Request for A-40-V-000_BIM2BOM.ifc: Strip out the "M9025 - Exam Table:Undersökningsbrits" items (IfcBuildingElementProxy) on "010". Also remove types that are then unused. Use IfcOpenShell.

First a look at what the model holds.

```python
import ifcopenshell
import ifcopenshell.util.element

model = ifcopenshell.open("A-40-V-000_BIM2BOM.ifc")
print(model.schema)
storey = next(s for s in model.by_type("IfcBuildingStorey") if s.Name == "010")
proxies = [e for e in ifcopenshell.util.element.get_decomposition(storey) if e.is_a("IfcBuildingElementProxy")]
seen = {}
for e in proxies:
    element_type = ifcopenshell.util.element.get_type(e)
    name = element_type.Name if element_type not in (None, e) else None
    seen[name] = seen.get(name, 0) + 1
for name, count in sorted(seen.items(), key=str):
    print(count, "x", name)
```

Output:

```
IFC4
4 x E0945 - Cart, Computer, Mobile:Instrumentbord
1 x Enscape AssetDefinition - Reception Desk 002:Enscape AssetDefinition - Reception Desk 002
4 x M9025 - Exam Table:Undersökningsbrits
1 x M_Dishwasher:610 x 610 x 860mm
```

```python
import ifcopenshell
import ifcopenshell.api.root
import ifcopenshell.util.element

model = ifcopenshell.open("A-40-V-000_BIM2BOM.ifc")

storey = next(s for s in model.by_type("IfcBuildingStorey") if s.Name == "010")
proxies = [e for e in ifcopenshell.util.element.get_decomposition(storey) if e.is_a("IfcBuildingElementProxy")]
targets = [e for e in proxies if (t := ifcopenshell.util.element.get_type(e)) not in (None, e) and t.Name == "M9025 - Exam Table:Undersökningsbrits"]
types = {ifcopenshell.util.element.get_type(e) for e in targets} - {None, *targets}

for e in targets:
    ifcopenshell.api.root.remove_product(model, product=e)
print(len(targets), "removed")

unused = [t for t in types if not ifcopenshell.util.element.get_types(t)]
for t in unused:
    ifcopenshell.api.root.remove_product(model, product=t)
print(len(unused), "unused types removed")

model.write("A-40-V-000_BIM2BOM_v2.ifc")
```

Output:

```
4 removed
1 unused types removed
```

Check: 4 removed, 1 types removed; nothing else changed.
